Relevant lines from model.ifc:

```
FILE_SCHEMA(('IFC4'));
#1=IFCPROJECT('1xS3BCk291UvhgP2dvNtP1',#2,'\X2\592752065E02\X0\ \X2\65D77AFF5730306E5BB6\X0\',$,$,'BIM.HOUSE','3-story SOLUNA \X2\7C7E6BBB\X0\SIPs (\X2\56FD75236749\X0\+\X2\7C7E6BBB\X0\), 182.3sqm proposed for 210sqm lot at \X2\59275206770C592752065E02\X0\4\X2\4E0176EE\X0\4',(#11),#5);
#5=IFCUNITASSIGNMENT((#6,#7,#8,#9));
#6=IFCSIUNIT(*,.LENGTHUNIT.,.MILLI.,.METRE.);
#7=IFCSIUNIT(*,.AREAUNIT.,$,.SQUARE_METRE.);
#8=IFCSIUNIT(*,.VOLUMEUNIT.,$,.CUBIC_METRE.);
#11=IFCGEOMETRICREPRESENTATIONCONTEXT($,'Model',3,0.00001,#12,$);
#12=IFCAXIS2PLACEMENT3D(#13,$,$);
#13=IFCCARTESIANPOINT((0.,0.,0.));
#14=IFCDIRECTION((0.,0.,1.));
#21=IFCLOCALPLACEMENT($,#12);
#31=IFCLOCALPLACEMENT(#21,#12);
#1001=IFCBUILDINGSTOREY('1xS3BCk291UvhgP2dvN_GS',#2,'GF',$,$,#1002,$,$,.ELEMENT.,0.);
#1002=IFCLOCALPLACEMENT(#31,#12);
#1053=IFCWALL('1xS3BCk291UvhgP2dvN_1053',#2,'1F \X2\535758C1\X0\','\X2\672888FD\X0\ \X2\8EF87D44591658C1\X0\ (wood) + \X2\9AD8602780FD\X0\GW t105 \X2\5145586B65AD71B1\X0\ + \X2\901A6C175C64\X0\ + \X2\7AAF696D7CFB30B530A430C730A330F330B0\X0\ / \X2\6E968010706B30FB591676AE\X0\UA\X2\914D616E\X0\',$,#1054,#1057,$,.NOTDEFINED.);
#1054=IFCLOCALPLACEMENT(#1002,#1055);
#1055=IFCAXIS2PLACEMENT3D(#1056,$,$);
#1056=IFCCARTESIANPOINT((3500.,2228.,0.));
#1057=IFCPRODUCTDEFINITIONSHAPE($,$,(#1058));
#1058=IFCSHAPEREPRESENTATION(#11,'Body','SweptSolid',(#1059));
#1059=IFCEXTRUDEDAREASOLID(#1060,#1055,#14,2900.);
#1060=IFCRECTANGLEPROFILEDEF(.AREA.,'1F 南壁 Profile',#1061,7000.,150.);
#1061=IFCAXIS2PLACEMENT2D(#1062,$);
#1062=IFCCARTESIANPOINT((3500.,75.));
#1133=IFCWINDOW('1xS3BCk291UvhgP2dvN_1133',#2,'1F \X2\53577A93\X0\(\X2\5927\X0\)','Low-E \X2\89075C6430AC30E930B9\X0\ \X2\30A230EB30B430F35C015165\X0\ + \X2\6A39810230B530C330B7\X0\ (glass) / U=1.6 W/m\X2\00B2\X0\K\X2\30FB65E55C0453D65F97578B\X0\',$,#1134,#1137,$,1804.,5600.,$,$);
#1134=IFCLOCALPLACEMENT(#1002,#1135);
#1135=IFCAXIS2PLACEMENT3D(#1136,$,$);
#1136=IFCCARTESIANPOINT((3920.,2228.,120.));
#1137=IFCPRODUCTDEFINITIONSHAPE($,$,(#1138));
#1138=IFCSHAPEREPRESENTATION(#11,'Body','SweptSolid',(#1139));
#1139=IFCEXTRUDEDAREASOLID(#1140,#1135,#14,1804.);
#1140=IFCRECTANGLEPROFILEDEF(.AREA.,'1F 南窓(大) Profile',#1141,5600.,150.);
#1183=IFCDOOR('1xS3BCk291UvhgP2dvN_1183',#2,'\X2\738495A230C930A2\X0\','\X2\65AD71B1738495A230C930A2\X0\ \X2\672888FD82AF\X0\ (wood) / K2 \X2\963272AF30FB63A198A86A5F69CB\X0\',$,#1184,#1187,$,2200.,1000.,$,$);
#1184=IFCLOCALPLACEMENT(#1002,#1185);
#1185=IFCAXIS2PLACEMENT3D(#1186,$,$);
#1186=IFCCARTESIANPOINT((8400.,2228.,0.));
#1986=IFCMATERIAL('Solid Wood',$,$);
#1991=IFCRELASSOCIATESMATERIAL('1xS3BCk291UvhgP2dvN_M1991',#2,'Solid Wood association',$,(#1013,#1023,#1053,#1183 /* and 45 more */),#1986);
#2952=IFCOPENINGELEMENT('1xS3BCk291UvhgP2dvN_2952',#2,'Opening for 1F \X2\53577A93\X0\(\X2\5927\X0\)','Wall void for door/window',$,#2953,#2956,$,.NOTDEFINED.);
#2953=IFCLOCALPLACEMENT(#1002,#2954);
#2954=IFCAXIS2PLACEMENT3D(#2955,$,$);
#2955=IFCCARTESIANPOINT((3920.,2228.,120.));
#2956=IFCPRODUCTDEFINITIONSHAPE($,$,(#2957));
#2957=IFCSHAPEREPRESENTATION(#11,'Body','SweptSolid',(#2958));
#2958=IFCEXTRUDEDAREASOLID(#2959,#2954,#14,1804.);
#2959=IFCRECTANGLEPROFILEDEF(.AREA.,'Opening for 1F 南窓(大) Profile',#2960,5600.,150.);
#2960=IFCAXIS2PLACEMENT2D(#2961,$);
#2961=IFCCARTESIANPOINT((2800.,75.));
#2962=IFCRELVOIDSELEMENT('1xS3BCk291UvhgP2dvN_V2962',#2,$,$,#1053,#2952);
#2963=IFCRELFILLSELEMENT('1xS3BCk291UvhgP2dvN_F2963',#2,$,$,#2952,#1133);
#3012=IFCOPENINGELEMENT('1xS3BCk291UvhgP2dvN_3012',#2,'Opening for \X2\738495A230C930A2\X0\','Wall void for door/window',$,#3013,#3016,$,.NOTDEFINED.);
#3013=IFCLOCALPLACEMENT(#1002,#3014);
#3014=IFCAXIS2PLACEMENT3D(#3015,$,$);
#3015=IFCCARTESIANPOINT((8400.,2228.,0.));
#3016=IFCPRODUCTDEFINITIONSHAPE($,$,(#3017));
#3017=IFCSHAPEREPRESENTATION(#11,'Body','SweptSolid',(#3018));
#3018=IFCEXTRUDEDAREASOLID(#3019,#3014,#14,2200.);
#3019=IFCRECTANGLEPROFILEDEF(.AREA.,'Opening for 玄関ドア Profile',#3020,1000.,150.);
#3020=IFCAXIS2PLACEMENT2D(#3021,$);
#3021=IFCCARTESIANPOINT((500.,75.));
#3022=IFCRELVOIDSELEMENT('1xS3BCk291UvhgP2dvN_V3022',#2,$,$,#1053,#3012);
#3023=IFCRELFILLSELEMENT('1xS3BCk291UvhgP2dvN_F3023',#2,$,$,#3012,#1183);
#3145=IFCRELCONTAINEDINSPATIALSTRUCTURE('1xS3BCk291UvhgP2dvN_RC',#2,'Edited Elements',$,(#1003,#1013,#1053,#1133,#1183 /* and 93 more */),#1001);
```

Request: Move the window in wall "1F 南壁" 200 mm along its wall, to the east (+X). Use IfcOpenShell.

```python
import ifcopenshell
import ifcopenshell.api.geometry
import ifcopenshell.util.placement
import ifcopenshell.util.unit

model = ifcopenshell.open("model.ifc")
unit_scale = ifcopenshell.util.unit.calculate_unit_scale(model)

window = model.by_id(1133)
opening = window.FillsVoids[0].RelatingOpeningElement
wall = opening.VoidsElements[0].RelatingBuildingElement

wall_matrix = ifcopenshell.util.placement.get_local_placement(wall.ObjectPlacement)
shift = wall_matrix[:3, 0] * 0.2 / unit_scale
before = ifcopenshell.util.placement.get_local_placement(window.ObjectPlacement)[:3, 3].copy()

# The window is not placed relative to its opening, so move both.
for product in (opening, window):
    matrix = ifcopenshell.util.placement.get_local_placement(product.ObjectPlacement)
    matrix[:3, 3] += shift
    ifcopenshell.api.geometry.edit_object_placement(model, product=product, matrix=matrix, is_si=False)

after = ifcopenshell.util.placement.get_local_placement(window.ObjectPlacement)[:3, 3]
print("window moved by", (after - before).round(3) + 0.0)

model.write("model_edited.ifc")
```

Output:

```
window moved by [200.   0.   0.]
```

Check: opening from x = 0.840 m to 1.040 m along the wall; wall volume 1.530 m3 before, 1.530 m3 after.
